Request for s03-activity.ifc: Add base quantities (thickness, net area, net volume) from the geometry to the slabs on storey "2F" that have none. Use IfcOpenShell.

First a look at what the model holds.

```python
import ifcopenshell
import ifcopenshell.util.element
import ifcopenshell.util.unit

model = ifcopenshell.open("s03-activity.ifc")
print(model.schema)
for unit_type in ("LENGTHUNIT", "AREAUNIT", "VOLUMEUNIT"):
    print(unit_type, ifcopenshell.util.unit.calculate_unit_scale(model, unit_type))
storey = next(s for s in model.by_type("IfcBuildingStorey") if s.Name == "2F")
slabs = [e for e in ifcopenshell.util.element.get_decomposition(storey) if e.is_a("IfcSlab")]
for e in sorted(slabs, key=lambda e: e.id()):
    print(e.id(), e.is_a(), e.Name, list(ifcopenshell.util.element.get_psets(e, qtos_only=True)), sep=" | ")
```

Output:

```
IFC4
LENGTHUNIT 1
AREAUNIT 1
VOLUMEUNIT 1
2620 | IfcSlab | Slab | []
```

```python
import ifcopenshell
import ifcopenshell.api.pset
import ifcopenshell.geom
import ifcopenshell.util.element
import ifcopenshell.util.shape
import ifcopenshell.util.unit

model = ifcopenshell.open("s03-activity.ifc")
unit_scale = ifcopenshell.util.unit.calculate_unit_scale(model)
area_scale = ifcopenshell.util.unit.calculate_unit_scale(model, "AREAUNIT")
volume_scale = ifcopenshell.util.unit.calculate_unit_scale(model, "VOLUMEUNIT")
settings = ifcopenshell.geom.settings()

storey = next(s for s in model.by_type("IfcBuildingStorey") if s.Name == "2F")
slabs = [e for e in ifcopenshell.util.element.get_decomposition(storey) if e.is_a("IfcSlab")]

for e in sorted(slabs, key=lambda e: e.id()):
    if ifcopenshell.util.element.get_psets(e, qtos_only=True, should_inherit=False):
        continue
    # Geometry comes back in metres, in the element's own axes.
    shape = ifcopenshell.geom.create_shape(settings, e)
    values = {
        "Width": ifcopenshell.util.shape.get_z(shape.geometry) / unit_scale,
        "NetArea": ifcopenshell.util.shape.get_footprint_area(shape.geometry) / area_scale,
        "NetVolume": ifcopenshell.util.shape.get_volume(shape.geometry) / volume_scale,
    }
    qto = ifcopenshell.api.pset.add_qto(model, product=e, name="Qto_SlabBaseQuantities")
    ifcopenshell.api.pset.edit_qto(model, qto=qto, properties=values)
    print(e.id(), {k: round(v, 3) for k, v in values.items()})

model.write("s03-activity_v2.ifc")
```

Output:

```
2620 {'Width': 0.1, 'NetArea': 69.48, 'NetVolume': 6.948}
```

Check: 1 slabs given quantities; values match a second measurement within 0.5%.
